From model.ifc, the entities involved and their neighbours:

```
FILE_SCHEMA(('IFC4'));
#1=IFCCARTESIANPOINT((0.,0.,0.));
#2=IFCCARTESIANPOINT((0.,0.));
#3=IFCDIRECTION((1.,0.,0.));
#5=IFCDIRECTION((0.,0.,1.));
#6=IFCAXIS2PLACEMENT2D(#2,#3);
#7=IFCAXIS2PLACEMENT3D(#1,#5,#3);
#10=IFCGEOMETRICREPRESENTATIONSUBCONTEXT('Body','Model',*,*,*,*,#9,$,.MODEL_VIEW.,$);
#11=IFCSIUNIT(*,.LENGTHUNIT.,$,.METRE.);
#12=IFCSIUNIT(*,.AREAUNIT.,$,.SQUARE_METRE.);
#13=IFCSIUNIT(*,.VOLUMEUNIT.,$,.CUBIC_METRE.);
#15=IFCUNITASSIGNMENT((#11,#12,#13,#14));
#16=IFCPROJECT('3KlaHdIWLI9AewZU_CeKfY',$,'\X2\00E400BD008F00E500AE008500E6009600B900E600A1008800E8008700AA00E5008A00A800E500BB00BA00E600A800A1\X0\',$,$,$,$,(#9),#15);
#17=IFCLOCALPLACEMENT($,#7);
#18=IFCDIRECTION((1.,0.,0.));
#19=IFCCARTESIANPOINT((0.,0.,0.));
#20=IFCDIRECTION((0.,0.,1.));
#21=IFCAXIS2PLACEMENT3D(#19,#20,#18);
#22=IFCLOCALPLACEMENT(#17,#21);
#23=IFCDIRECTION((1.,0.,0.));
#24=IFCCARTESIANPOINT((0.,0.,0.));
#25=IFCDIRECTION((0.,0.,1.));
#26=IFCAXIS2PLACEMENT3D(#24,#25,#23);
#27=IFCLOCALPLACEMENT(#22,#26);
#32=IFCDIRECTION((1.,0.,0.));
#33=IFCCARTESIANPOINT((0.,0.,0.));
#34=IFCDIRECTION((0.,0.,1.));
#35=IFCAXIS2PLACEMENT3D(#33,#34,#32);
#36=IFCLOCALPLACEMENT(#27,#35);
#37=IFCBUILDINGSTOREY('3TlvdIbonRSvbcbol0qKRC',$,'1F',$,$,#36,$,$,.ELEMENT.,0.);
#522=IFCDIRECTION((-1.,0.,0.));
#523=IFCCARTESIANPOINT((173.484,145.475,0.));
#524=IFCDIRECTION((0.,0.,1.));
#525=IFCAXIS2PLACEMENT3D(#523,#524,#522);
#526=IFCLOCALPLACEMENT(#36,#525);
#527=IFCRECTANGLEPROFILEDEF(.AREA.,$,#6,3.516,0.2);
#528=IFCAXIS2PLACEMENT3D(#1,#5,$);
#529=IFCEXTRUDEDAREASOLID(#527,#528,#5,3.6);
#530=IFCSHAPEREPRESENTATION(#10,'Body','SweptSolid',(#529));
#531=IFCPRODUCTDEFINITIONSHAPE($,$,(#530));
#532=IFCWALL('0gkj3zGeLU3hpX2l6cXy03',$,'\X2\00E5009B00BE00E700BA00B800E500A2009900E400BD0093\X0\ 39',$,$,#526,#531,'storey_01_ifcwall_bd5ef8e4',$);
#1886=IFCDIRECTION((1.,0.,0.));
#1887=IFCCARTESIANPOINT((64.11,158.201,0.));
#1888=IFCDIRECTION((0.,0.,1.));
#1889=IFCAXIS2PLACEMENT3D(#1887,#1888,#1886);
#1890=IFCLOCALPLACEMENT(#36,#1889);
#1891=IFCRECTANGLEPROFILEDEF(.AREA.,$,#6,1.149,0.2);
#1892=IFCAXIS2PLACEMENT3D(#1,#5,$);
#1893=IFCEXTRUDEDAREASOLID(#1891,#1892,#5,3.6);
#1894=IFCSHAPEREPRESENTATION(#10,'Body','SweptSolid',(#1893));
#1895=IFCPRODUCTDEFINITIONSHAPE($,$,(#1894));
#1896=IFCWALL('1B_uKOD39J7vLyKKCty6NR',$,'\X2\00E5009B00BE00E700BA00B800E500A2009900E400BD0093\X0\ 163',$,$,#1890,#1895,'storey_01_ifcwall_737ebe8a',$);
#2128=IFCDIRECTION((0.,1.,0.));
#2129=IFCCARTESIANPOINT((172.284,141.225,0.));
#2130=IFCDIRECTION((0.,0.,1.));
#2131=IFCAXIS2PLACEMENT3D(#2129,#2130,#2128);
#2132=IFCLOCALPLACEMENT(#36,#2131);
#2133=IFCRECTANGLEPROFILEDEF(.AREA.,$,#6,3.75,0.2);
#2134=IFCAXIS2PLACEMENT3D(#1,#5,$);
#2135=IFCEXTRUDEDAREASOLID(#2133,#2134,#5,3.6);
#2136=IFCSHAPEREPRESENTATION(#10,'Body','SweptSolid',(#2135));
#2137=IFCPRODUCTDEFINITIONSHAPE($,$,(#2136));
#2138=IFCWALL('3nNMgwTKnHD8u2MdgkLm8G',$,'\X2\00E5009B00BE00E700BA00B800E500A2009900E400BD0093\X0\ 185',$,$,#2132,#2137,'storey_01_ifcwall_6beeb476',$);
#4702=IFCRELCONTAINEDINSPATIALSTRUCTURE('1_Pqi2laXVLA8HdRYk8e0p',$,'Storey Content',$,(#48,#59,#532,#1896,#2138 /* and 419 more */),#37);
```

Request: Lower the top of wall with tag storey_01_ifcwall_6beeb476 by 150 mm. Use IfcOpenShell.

```python
import ifcopenshell
import ifcopenshell.geom
import ifcopenshell.util.representation
import ifcopenshell.util.shape
import ifcopenshell.util.unit

model = ifcopenshell.open("model.ifc")
unit_scale = ifcopenshell.util.unit.calculate_unit_scale(model)
settings = ifcopenshell.geom.settings()


def volume(element):
    """Net volume in cubic metres, openings subtracted."""
    shape = ifcopenshell.geom.create_shape(settings, element)
    return ifcopenshell.util.shape.get_volume(shape.geometry)


wall = model.by_guid("3nNMgwTKnHD8u2MdgkLm8G")
before = volume(wall)

body = ifcopenshell.util.representation.get_representation(wall, "Model", "Body")
solid = body.Items[0]
old_height = solid.Depth
solid.Depth -= 0.15 / unit_scale
after = volume(wall)

print(f"height {old_height:g} -> {solid.Depth:g}, volume {before:.3f} -> {after:.3f} m3")

model.write("model_rev.ifc")
```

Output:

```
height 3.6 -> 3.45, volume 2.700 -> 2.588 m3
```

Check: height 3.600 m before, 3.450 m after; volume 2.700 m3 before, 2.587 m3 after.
